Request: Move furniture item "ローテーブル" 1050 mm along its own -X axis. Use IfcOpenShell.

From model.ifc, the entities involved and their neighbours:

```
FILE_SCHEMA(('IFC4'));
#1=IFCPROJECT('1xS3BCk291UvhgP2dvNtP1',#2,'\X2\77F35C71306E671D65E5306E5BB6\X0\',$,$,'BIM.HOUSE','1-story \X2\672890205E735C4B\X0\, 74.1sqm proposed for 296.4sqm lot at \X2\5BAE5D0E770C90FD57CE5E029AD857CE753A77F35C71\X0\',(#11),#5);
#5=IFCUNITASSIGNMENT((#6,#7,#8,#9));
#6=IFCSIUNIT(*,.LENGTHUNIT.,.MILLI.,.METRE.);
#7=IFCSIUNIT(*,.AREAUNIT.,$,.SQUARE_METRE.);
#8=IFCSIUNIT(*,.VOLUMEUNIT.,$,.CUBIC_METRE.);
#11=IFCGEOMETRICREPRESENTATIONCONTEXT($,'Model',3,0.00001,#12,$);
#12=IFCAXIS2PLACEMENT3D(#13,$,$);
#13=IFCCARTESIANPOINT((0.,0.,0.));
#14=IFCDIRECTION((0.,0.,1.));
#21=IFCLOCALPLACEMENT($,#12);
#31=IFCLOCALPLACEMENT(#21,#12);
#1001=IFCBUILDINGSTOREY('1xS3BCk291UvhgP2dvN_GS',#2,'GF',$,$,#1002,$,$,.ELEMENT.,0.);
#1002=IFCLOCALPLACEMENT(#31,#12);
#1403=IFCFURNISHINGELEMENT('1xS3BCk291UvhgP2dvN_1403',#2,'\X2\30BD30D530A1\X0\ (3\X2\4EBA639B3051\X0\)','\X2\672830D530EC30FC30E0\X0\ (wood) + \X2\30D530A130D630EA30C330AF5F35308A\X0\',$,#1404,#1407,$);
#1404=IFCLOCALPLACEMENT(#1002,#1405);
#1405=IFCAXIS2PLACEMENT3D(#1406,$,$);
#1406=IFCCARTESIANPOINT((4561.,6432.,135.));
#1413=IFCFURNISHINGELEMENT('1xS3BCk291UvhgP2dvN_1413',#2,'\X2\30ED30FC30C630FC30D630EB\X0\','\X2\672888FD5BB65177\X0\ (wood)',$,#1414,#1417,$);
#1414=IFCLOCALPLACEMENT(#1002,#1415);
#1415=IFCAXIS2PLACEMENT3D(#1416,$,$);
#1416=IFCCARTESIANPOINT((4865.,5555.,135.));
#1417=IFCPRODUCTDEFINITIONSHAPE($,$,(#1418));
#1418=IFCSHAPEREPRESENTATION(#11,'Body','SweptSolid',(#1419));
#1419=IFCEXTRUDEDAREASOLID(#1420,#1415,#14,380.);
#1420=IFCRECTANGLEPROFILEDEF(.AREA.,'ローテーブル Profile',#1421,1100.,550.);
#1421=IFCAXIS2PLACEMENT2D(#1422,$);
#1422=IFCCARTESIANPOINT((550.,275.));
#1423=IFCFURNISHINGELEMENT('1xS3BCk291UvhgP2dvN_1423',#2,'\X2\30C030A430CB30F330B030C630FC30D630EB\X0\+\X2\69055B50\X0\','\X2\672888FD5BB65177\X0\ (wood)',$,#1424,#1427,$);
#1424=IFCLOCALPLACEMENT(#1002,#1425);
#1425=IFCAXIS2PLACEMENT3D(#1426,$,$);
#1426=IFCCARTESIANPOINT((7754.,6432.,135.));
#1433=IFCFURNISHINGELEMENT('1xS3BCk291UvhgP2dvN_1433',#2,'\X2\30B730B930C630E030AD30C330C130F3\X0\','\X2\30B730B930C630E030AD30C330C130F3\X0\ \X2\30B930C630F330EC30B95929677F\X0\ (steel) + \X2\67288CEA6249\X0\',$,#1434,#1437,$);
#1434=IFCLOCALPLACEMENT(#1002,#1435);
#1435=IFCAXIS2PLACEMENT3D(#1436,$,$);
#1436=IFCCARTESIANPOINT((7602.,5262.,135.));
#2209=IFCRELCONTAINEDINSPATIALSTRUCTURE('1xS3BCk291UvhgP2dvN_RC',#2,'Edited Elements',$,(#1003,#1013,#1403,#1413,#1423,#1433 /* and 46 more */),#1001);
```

```python
import ifcopenshell
import ifcopenshell.api.geometry
import ifcopenshell.util.placement

model = ifcopenshell.open("model.ifc")

item = model.by_guid("1xS3BCk291UvhgP2dvN_1413")
matrix = ifcopenshell.util.placement.get_local_placement(item.ObjectPlacement)
matrix[:3, 3] -= matrix[:3, 0] * 1050.0
ifcopenshell.api.geometry.edit_object_placement(model, product=item, matrix=matrix, is_si=False)

print(ifcopenshell.util.placement.get_local_placement(item.ObjectPlacement).round(3) + 0.0)

model.write("model-out.ifc")
```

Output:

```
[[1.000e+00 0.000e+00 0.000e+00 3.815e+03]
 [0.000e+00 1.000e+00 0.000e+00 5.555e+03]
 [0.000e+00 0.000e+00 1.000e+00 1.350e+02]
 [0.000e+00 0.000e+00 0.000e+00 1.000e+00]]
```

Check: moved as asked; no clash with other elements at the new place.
